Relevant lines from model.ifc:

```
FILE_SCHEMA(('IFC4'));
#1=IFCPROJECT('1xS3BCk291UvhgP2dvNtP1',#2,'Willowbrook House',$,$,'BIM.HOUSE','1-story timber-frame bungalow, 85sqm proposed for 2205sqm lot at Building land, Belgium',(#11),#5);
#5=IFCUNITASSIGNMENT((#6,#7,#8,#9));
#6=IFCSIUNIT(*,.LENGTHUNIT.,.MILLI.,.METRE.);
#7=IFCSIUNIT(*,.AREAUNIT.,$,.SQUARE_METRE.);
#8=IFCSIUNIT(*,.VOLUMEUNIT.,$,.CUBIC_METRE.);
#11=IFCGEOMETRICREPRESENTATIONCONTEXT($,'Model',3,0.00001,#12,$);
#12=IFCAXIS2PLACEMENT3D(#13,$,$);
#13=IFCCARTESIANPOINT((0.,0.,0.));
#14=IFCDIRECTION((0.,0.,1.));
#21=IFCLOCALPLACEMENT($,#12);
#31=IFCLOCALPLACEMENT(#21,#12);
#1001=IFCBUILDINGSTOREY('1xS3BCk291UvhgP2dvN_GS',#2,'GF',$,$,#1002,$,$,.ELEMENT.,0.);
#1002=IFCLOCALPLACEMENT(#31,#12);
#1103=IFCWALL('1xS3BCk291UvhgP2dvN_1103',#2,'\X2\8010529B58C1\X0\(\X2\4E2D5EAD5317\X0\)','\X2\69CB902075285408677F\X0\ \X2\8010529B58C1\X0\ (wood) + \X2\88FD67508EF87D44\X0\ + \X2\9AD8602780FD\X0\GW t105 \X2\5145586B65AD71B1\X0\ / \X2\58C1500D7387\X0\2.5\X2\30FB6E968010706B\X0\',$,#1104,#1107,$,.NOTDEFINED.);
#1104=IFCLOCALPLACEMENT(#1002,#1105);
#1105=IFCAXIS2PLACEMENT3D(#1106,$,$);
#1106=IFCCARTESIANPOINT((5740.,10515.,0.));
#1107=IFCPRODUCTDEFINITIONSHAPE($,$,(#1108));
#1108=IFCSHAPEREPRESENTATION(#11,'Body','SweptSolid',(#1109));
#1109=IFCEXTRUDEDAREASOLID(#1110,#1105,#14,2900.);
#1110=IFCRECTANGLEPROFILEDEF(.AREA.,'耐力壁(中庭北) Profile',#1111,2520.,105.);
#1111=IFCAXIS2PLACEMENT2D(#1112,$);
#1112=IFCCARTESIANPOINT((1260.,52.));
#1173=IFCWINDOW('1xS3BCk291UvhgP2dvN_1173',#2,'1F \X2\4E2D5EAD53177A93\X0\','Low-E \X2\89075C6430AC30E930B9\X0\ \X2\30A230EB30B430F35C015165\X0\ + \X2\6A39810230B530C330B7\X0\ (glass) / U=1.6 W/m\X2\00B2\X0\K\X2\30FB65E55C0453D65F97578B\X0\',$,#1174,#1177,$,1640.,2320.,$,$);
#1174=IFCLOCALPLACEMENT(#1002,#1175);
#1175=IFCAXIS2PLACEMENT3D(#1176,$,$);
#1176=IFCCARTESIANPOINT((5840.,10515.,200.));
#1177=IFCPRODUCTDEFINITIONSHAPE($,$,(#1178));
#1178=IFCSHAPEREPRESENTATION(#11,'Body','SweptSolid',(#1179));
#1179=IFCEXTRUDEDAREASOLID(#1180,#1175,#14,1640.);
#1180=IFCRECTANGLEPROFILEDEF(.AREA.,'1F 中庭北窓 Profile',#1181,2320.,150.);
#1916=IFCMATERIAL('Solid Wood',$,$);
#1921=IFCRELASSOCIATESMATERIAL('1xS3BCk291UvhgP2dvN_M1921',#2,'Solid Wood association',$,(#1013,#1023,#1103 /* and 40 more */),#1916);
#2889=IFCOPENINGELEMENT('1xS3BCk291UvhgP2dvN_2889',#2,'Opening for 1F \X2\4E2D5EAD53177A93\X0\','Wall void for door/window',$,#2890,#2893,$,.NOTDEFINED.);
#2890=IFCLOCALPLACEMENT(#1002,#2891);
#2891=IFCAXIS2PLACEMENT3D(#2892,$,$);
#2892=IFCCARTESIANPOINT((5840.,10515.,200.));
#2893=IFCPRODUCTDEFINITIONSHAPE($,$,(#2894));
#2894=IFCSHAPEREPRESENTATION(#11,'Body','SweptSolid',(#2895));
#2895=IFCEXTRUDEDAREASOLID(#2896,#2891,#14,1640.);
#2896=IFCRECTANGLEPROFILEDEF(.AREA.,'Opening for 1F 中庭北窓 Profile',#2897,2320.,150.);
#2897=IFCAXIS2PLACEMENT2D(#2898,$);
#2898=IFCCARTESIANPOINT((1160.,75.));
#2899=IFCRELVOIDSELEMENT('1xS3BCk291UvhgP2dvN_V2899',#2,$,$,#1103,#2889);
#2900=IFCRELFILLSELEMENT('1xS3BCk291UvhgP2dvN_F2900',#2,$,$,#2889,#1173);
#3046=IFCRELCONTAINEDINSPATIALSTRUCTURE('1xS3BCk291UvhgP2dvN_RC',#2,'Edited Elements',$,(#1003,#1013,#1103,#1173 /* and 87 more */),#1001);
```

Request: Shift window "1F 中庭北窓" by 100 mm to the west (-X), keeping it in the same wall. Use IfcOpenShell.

```python
import ifcopenshell
import ifcopenshell.api.geometry
import ifcopenshell.util.placement
import ifcopenshell.util.unit

model = ifcopenshell.open("model.ifc")
unit_scale = ifcopenshell.util.unit.calculate_unit_scale(model)

window = model.by_id(1173)
opening = window.FillsVoids[0].RelatingOpeningElement
wall = opening.VoidsElements[0].RelatingBuildingElement

wall_matrix = ifcopenshell.util.placement.get_local_placement(wall.ObjectPlacement)
shift = wall_matrix[:3, 0] * -0.1 / unit_scale
before = ifcopenshell.util.placement.get_local_placement(window.ObjectPlacement)[:3, 3].copy()

# The window is not placed relative to its opening, so move both.
for product in (opening, window):
    matrix = ifcopenshell.util.placement.get_local_placement(product.ObjectPlacement)
    matrix[:3, 3] += shift
    ifcopenshell.api.geometry.edit_object_placement(model, product=product, matrix=matrix, is_si=False)

after = ifcopenshell.util.placement.get_local_placement(window.ObjectPlacement)[:3, 3]
print("window moved by", (after - before).round(3) + 0.0)

model.write("model_edited.ifc")
```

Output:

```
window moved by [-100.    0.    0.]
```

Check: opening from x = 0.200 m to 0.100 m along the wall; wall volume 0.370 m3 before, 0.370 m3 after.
